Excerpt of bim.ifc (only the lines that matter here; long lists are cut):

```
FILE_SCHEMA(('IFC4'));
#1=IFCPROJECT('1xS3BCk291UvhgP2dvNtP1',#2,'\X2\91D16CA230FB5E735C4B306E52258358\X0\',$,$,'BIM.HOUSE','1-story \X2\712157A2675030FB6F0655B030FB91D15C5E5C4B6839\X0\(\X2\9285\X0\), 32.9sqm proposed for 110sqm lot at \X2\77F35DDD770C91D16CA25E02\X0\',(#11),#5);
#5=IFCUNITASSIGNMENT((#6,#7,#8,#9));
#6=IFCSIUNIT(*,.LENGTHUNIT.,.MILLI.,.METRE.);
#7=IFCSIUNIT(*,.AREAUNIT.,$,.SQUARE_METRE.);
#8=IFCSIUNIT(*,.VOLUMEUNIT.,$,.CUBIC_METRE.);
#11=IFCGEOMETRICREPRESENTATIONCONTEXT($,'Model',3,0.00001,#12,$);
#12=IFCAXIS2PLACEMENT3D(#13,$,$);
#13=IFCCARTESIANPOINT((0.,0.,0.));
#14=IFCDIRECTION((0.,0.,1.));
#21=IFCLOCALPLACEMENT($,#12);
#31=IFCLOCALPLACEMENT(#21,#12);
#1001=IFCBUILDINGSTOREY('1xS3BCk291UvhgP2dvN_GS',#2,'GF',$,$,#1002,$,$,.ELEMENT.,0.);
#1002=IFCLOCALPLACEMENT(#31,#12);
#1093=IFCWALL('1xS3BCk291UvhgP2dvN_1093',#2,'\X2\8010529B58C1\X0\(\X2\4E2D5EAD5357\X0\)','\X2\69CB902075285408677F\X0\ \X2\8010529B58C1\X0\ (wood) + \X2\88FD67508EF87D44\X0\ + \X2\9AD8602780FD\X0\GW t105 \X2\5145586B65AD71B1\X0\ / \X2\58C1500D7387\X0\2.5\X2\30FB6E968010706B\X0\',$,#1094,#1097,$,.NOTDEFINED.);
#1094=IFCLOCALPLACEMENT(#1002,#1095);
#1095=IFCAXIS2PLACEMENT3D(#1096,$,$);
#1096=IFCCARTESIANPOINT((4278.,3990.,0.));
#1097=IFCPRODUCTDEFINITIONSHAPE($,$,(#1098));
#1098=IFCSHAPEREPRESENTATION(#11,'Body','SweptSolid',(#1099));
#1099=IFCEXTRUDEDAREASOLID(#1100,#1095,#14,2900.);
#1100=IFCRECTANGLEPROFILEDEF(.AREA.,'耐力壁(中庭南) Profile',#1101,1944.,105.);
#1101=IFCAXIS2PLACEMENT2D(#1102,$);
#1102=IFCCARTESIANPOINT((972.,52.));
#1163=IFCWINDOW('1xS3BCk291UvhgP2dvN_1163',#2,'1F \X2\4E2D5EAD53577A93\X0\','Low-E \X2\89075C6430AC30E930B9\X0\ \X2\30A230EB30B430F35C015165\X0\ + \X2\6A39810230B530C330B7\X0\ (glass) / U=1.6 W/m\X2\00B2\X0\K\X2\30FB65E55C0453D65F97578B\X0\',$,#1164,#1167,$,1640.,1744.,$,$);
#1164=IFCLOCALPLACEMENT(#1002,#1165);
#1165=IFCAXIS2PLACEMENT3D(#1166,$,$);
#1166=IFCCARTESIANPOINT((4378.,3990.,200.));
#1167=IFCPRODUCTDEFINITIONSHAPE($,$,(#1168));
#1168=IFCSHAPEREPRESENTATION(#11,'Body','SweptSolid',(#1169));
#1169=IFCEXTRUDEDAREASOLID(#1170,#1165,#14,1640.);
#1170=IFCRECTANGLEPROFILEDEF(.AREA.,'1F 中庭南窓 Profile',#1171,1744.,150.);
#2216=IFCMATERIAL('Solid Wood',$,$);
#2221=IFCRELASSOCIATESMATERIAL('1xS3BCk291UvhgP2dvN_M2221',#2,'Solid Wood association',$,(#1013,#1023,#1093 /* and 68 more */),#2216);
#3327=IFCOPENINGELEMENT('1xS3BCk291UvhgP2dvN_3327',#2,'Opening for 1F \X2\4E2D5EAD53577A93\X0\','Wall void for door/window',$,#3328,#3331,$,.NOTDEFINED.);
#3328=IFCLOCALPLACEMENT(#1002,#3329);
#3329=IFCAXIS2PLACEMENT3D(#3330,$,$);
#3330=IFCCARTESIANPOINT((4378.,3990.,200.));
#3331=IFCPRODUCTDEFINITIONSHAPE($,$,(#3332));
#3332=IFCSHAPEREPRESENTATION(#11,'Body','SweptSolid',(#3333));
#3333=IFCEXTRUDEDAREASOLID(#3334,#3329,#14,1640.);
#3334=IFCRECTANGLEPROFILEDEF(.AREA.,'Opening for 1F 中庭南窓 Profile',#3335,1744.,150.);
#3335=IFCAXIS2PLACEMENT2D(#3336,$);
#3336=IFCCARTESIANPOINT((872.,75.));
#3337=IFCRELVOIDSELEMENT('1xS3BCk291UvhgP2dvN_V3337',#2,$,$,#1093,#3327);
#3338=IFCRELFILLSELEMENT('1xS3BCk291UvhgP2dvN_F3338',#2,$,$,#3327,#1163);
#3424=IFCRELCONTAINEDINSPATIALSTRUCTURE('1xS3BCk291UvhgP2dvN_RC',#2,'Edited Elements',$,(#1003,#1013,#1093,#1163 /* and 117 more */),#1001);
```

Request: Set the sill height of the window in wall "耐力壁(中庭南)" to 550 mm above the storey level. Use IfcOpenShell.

```python
import numpy as np
import ifcopenshell
import ifcopenshell.api.geometry
import ifcopenshell.geom
import ifcopenshell.util.element
import ifcopenshell.util.placement
import ifcopenshell.util.shape
import ifcopenshell.util.unit

model = ifcopenshell.open("bim.ifc")
unit_scale = ifcopenshell.util.unit.calculate_unit_scale(model)

window = model.by_guid("1xS3BCk291UvhgP2dvN_1163")
opening = window.FillsVoids[0].RelatingOpeningElement
storey = ifcopenshell.util.element.get_container(window, ifc_class="IfcBuildingStorey")
level = ifcopenshell.util.placement.get_local_placement(storey.ObjectPlacement)[2, 3]

# The opening's origin need not be at the sill, so measure its lowest point.
shape = ifcopenshell.geom.create_shape(ifcopenshell.geom.settings(), opening)
bottom = ifcopenshell.util.shape.get_shape_bottom_elevation(shape, shape.geometry) / unit_scale
dz = level + 0.55 / unit_scale - bottom

shift = np.array([0.0, 0.0, dz])
# The window is not placed relative to its opening, so move both.
for product in (opening, window):
    matrix = ifcopenshell.util.placement.get_local_placement(product.ObjectPlacement)
    matrix[:3, 3] += shift
    ifcopenshell.api.geometry.edit_object_placement(model, product=product, matrix=matrix, is_si=False)

print(f"moved by {dz * unit_scale:+.3f} m")

model.write("bim_updated.ifc")
```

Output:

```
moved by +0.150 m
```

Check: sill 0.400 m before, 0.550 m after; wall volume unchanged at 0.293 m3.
